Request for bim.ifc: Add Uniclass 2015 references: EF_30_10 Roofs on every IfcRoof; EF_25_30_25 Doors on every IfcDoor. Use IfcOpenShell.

First a look at what the model holds.

```python
import ifcopenshell

model = ifcopenshell.open("bim.ifc")
print(model.schema)
print("classifications:", [c.Name for c in model.by_type("IfcClassification")])
for ifc_class in ("IfcDoor", "IfcRoof", "IfcStair", "IfcWall", "IfcWindow"):
    print(ifc_class, len(model.by_type(ifc_class)))
```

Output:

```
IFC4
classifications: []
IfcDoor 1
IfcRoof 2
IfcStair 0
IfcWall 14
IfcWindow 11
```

```python
import ifcopenshell
import ifcopenshell.api.classification

model = ifcopenshell.open("bim.ifc")

system = ifcopenshell.api.classification.add_classification(model, classification="Uniclass 2015")

codes = {
    "IfcRoof": ("EF_30_10", "Roofs"),
    "IfcDoor": ("EF_25_30_25", "Doors"),
}
for ifc_class, (code, name) in codes.items():
    products = model.by_type(ifc_class)
    ifcopenshell.api.classification.add_reference(
        model, products=products, classification=system, identification=code, name=name
    )
    print(code, len(products))

model.write("bim_rev.ifc")
```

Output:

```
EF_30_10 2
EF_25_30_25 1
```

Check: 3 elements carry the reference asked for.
